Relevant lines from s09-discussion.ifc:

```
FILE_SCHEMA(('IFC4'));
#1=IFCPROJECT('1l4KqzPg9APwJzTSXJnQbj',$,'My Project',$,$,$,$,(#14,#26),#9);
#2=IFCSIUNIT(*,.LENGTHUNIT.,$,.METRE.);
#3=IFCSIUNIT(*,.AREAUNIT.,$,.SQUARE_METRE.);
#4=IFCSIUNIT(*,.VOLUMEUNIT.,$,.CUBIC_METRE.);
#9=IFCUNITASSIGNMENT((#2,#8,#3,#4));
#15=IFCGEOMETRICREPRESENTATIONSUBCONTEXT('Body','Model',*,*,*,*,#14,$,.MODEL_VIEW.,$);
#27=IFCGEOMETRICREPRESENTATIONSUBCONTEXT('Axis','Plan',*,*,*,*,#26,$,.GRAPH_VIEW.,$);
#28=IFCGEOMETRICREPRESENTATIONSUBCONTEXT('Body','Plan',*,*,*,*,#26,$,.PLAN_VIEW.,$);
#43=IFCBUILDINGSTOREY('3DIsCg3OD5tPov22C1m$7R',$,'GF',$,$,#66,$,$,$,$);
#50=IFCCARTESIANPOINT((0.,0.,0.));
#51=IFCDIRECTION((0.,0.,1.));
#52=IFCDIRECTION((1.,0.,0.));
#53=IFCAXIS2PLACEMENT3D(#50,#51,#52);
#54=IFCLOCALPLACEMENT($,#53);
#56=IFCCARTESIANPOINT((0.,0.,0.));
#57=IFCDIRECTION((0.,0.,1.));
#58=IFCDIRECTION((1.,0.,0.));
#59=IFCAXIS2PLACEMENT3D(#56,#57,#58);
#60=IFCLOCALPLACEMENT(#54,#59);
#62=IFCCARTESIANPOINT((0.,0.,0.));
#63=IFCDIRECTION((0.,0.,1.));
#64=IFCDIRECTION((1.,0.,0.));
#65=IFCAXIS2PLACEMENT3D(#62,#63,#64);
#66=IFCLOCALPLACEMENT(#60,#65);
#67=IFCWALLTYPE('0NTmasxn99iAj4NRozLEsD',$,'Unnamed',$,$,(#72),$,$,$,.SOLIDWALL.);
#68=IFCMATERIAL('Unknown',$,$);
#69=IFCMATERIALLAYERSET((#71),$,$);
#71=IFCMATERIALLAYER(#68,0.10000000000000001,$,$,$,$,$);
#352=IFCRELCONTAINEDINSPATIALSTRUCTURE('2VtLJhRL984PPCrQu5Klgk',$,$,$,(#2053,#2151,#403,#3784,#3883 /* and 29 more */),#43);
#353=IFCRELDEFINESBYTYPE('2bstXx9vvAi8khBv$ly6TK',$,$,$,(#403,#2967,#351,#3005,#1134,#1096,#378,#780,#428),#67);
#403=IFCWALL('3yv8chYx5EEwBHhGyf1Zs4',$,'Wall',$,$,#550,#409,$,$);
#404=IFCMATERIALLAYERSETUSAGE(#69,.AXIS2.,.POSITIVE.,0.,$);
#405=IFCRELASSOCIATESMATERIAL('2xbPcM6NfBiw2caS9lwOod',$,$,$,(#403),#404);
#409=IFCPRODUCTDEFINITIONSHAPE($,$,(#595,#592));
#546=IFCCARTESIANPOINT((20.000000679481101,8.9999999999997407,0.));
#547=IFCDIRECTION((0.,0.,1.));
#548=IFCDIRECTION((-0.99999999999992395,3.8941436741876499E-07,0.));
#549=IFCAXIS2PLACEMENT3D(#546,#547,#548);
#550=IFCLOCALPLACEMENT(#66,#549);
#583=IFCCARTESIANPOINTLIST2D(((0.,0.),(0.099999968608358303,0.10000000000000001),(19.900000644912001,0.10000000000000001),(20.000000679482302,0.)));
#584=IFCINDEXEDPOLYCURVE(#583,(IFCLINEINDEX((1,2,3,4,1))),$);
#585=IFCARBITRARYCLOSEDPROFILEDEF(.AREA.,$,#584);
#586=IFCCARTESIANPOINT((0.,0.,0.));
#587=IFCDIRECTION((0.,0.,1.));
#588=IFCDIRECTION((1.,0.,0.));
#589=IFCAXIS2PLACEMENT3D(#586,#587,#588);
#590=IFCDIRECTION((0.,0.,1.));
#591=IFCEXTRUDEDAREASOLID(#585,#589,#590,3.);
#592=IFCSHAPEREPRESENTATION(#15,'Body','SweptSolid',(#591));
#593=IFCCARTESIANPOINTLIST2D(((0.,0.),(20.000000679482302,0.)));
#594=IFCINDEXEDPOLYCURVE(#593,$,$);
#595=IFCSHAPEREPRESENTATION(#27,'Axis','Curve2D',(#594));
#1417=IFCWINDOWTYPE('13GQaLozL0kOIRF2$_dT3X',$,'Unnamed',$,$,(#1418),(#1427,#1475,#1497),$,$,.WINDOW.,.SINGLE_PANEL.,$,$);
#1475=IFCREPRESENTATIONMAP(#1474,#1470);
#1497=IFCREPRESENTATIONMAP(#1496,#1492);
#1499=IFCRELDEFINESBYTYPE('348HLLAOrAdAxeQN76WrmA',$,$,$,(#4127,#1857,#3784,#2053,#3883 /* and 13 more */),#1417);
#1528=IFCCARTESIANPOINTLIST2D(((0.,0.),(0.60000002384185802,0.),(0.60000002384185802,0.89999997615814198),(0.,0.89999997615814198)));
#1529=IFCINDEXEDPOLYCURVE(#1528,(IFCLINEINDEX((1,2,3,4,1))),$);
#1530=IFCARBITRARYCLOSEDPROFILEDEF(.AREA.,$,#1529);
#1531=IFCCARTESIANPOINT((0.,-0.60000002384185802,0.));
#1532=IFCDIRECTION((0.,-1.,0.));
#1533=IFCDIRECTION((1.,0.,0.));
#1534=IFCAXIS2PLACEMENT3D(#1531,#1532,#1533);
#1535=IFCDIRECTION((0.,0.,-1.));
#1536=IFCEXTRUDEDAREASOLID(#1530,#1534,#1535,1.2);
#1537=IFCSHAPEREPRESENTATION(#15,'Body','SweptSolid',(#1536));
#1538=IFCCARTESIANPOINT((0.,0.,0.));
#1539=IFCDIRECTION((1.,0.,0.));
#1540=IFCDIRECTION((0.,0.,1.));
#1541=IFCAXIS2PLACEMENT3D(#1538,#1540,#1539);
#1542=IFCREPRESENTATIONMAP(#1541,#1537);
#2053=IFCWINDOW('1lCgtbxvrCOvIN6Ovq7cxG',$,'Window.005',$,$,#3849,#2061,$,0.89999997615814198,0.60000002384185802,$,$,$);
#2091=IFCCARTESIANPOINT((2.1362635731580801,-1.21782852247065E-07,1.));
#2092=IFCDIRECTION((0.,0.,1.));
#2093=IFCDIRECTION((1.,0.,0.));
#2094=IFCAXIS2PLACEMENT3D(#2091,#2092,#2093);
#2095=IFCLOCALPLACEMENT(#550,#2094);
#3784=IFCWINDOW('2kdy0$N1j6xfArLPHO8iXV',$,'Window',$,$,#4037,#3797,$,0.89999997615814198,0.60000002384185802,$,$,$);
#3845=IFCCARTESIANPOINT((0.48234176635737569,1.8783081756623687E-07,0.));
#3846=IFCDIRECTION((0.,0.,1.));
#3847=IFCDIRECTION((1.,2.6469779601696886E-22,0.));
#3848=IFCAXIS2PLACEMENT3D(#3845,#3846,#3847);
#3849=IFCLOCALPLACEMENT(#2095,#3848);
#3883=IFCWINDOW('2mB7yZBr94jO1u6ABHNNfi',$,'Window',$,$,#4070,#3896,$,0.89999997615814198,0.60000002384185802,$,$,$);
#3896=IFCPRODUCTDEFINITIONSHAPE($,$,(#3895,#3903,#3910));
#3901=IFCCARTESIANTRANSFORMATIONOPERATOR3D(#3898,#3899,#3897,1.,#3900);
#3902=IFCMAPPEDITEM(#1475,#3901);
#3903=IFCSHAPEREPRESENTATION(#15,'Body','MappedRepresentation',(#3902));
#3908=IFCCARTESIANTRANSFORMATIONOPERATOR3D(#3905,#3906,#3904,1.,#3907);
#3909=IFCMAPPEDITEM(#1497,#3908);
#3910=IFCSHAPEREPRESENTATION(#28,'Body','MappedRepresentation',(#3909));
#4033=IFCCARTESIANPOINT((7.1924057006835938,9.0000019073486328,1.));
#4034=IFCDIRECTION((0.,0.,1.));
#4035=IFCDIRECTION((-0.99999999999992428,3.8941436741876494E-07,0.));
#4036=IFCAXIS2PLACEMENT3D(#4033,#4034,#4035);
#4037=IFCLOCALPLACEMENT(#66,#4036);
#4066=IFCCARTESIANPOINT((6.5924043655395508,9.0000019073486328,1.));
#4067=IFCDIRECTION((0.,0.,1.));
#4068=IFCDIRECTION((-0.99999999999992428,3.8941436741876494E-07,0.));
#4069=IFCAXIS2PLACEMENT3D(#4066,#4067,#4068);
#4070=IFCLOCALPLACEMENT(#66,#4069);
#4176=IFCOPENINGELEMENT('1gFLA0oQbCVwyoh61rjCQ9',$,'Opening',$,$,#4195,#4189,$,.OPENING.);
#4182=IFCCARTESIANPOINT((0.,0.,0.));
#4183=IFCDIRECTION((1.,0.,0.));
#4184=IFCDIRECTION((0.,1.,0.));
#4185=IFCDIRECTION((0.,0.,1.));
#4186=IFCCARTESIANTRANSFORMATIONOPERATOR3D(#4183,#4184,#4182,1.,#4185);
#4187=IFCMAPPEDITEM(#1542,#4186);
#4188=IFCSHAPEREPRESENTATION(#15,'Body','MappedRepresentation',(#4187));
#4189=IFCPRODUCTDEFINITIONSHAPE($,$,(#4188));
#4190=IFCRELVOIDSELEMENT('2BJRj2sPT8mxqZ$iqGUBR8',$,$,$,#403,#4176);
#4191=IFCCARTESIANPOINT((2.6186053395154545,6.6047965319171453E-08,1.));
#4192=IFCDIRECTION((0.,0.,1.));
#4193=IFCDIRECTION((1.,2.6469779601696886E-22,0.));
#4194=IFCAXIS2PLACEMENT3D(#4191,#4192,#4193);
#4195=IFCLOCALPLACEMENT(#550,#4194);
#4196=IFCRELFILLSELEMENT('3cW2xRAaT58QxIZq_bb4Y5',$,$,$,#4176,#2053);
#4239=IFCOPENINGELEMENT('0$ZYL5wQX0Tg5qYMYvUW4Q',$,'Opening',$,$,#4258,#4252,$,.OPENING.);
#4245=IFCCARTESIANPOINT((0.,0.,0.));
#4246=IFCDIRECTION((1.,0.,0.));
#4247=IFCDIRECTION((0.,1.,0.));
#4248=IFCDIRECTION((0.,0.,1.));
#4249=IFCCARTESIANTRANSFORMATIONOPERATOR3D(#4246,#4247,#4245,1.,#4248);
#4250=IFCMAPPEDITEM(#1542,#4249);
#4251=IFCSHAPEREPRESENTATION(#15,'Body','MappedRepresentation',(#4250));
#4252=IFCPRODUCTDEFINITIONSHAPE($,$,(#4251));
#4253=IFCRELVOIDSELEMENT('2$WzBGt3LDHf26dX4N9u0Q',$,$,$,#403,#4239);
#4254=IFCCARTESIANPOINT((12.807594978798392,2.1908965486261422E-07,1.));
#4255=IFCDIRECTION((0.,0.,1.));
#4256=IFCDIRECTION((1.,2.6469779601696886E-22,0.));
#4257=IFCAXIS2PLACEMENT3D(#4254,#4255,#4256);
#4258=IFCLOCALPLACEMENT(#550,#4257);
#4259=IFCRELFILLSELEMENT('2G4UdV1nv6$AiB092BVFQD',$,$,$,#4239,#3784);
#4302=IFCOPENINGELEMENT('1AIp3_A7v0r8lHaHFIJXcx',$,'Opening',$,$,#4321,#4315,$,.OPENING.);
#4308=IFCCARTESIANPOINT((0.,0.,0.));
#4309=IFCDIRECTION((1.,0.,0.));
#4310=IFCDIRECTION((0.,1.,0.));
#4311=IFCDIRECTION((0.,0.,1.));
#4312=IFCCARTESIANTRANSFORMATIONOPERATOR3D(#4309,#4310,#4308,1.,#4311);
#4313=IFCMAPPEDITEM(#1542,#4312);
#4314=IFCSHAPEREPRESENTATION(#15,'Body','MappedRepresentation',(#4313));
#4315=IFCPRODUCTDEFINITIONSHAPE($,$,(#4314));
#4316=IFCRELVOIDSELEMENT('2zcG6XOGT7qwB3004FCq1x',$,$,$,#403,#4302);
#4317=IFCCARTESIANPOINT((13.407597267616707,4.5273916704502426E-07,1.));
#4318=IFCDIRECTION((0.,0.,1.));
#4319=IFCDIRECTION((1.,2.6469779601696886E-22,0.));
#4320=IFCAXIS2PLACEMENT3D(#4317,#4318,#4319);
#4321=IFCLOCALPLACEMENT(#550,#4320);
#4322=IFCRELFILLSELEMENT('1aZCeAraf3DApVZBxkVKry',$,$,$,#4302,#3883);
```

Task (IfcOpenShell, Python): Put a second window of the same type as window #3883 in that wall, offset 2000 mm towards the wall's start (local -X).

```python
import ifcopenshell
import ifcopenshell.api.feature
import ifcopenshell.api.geometry
import ifcopenshell.api.root
import ifcopenshell.geom
import ifcopenshell.util.element
import ifcopenshell.util.placement
import ifcopenshell.util.shape

model = ifcopenshell.open("s09-discussion.ifc")
settings = ifcopenshell.geom.settings()


def volume(element):
    """Net volume in cubic metres, openings subtracted."""
    shape = ifcopenshell.geom.create_shape(settings, element)
    return ifcopenshell.util.shape.get_volume(shape.geometry)


window = model.by_guid("2mB7yZBr94jO1u6ABHNNfi")
opening = window.FillsVoids[0].RelatingOpeningElement
wall = opening.VoidsElements[0].RelatingBuildingElement
before = volume(wall)
shift = ifcopenshell.util.placement.get_local_placement(wall.ObjectPlacement)[:3, 0] * -2.0

# copy_class copies the void relationship, type, container and properties, but no geometry.
new_opening = ifcopenshell.api.root.copy_class(model, product=opening)
new_opening.Representation = ifcopenshell.util.element.copy_deep(
    model, opening.Representation, exclude=["IfcGeometricRepresentationContext", "IfcRepresentationMap"]
)
new_window = ifcopenshell.api.root.copy_class(model, product=window)
new_window.Representation = ifcopenshell.util.element.copy_deep(
    model, window.Representation, exclude=["IfcGeometricRepresentationContext", "IfcRepresentationMap"]
)
ifcopenshell.api.feature.add_filling(model, opening=new_opening, element=new_window)

for old, new in ((opening, new_opening), (window, new_window)):
    matrix = ifcopenshell.util.placement.get_local_placement(old.ObjectPlacement)
    matrix[:3, 3] += shift
    ifcopenshell.api.geometry.edit_object_placement(model, product=new, matrix=matrix, is_si=False)

after = volume(wall)

print(f"wall volume {before:.3f} -> {after:.3f} m3")

model.write("s09-discussion-out.ifc")
```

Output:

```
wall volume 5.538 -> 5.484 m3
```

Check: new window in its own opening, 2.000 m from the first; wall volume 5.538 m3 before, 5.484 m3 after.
